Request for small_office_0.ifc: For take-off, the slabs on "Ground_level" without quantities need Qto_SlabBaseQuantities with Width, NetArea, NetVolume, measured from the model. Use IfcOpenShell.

First a look at what the model holds.

```python
import ifcopenshell
import ifcopenshell.util.element
import ifcopenshell.util.unit

model = ifcopenshell.open("small_office_0.ifc")
print(model.schema)
for unit_type in ("LENGTHUNIT", "AREAUNIT", "VOLUMEUNIT"):
    print(unit_type, ifcopenshell.util.unit.calculate_unit_scale(model, unit_type))
storey = next(s for s in model.by_type("IfcBuildingStorey") if s.Name == "Ground_level")
slabs = [e for e in ifcopenshell.util.element.get_decomposition(storey) if e.is_a("IfcSlab")]
for e in sorted(slabs, key=lambda e: e.id()):
    print(e.id(), e.is_a(), e.Name, list(ifcopenshell.util.element.get_psets(e, qtos_only=True)), sep=" | ")
```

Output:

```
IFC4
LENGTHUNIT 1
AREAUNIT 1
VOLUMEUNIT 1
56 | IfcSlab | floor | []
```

```python
import ifcopenshell
import ifcopenshell.api.pset
import ifcopenshell.geom
import ifcopenshell.util.element
import ifcopenshell.util.shape
import ifcopenshell.util.unit

model = ifcopenshell.open("small_office_0.ifc")
unit_scale = ifcopenshell.util.unit.calculate_unit_scale(model)
area_scale = ifcopenshell.util.unit.calculate_unit_scale(model, "AREAUNIT")
volume_scale = ifcopenshell.util.unit.calculate_unit_scale(model, "VOLUMEUNIT")
settings = ifcopenshell.geom.settings()

storey = next(s for s in model.by_type("IfcBuildingStorey") if s.Name == "Ground_level")
slabs = [e for e in ifcopenshell.util.element.get_decomposition(storey) if e.is_a("IfcSlab")]

for e in sorted(slabs, key=lambda e: e.id()):
    if ifcopenshell.util.element.get_psets(e, qtos_only=True, should_inherit=False):
        continue
    # Geometry comes back in metres, in the element's own axes.
    shape = ifcopenshell.geom.create_shape(settings, e)
    values = {
        "Width": ifcopenshell.util.shape.get_z(shape.geometry) / unit_scale,
        "NetArea": ifcopenshell.util.shape.get_footprint_area(shape.geometry) / area_scale,
        "NetVolume": ifcopenshell.util.shape.get_volume(shape.geometry) / volume_scale,
    }
    qto = ifcopenshell.api.pset.add_qto(model, product=e, name="Qto_SlabBaseQuantities")
    ifcopenshell.api.pset.edit_qto(model, qto=qto, properties=values)
    print(e.id(), {k: round(v, 3) for k, v in values.items()})

model.write("small_office_0_v2.ifc")
```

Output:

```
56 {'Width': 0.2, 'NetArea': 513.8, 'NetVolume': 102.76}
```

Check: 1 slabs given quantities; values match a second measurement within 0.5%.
